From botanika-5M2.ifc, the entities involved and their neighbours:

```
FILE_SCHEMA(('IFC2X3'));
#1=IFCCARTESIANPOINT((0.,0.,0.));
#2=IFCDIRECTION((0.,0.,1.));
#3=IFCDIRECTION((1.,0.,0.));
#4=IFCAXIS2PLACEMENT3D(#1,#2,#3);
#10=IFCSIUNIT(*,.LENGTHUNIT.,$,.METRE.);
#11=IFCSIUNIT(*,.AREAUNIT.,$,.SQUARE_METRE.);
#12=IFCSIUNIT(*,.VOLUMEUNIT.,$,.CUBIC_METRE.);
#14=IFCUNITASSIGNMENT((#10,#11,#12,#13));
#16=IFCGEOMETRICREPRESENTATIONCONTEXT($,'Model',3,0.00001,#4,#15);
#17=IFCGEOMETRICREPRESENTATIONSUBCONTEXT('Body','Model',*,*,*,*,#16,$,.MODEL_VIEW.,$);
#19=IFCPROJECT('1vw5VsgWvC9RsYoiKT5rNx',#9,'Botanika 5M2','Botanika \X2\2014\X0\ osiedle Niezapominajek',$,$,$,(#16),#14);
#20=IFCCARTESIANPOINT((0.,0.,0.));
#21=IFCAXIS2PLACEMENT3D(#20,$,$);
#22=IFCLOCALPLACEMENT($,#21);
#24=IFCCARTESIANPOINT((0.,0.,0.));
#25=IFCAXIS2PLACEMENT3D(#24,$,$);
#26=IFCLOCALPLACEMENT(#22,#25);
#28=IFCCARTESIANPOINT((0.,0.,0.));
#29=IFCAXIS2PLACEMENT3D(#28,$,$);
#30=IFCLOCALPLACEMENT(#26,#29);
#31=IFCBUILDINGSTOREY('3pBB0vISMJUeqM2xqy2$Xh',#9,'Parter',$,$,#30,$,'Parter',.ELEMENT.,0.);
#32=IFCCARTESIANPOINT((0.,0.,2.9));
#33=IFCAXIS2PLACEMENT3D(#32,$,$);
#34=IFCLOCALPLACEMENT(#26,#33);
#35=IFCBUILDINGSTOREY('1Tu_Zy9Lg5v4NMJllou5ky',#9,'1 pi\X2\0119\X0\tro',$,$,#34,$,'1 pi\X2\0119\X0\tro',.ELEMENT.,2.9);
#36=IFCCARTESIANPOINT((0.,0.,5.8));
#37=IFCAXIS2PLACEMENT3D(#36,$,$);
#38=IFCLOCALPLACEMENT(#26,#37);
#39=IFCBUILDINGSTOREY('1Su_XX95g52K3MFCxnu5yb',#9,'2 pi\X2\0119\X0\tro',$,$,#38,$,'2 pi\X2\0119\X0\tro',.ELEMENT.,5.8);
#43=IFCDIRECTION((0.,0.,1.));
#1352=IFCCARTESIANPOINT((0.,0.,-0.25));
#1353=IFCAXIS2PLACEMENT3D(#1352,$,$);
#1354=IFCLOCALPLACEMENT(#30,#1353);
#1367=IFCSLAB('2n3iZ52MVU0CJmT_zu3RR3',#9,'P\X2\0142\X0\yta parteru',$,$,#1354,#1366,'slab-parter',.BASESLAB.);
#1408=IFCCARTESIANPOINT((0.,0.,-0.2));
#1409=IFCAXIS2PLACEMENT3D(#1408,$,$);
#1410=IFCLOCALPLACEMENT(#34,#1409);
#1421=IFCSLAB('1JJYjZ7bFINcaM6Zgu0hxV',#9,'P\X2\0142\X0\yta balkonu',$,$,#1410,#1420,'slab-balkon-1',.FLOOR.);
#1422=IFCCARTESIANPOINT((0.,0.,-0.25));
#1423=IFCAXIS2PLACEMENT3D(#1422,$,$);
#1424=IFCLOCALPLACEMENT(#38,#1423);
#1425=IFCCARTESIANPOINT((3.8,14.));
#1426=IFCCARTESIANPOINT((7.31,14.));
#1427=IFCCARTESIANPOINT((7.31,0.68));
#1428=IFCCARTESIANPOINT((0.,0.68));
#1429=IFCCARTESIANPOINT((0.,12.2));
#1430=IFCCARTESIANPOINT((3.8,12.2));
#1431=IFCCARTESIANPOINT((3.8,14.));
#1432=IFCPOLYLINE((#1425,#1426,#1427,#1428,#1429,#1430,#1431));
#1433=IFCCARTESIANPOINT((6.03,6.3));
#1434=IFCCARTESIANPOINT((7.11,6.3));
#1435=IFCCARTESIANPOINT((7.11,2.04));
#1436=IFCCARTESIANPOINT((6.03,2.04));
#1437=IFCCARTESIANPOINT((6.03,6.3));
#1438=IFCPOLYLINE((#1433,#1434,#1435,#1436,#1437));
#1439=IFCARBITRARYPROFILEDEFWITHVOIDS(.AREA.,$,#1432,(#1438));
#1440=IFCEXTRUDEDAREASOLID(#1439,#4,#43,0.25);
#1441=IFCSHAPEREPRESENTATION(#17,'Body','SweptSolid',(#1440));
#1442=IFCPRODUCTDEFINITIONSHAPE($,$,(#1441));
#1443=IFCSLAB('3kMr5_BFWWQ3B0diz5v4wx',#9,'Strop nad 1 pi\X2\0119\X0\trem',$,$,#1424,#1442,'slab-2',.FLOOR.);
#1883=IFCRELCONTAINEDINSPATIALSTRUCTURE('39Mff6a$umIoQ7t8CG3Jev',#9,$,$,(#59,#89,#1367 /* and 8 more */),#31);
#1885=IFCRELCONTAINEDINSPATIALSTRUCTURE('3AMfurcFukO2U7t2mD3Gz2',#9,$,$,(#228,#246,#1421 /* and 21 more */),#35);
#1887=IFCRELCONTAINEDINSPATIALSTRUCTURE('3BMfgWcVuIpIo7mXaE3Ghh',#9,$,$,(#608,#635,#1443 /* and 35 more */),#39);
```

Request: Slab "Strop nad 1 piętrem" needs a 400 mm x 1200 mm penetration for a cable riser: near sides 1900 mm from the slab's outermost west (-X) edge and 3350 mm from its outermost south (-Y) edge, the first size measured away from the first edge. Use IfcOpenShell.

```python
import numpy as np
import ifcopenshell
import ifcopenshell.api.feature
import ifcopenshell.api.geometry
import ifcopenshell.api.root
import ifcopenshell.geom
import ifcopenshell.util.placement
import ifcopenshell.util.representation
import ifcopenshell.util.shape
import ifcopenshell.util.unit

model = ifcopenshell.open("botanika-5M2.ifc")
unit_scale = ifcopenshell.util.unit.calculate_unit_scale(model)
settings = ifcopenshell.geom.settings()


def volume(element):
    """Net volume in cubic metres, openings subtracted."""
    shape = ifcopenshell.geom.create_shape(settings, element)
    return ifcopenshell.util.shape.get_volume(shape.geometry)


slab = model.by_guid("3kMr5_BFWWQ3B0diz5v4wx")
before = volume(slab)

# Extent in the slab's own axes, in metres. The edges named are its -X and -Y sides.
slab_shape = ifcopenshell.geom.create_shape(settings, slab)
vertices = ifcopenshell.util.shape.get_vertices(slab_shape.geometry)
x_min, y_min, bottom = vertices.min(axis=0)
top = vertices[:, 2].max()

opening = ifcopenshell.api.root.create_entity(model, ifc_class="IfcOpeningElement", name="Cable riser opening")
context = ifcopenshell.util.representation.get_context(model, "Model", "Body", "MODEL_VIEW")
width, depth = 0.4, 1.2
outline = [(0.0, 0.0), (width, 0.0), (width, depth), (0.0, depth), (0.0, 0.0)]
# Overshoot both faces by 50 mm so the cut is clean.
shape = ifcopenshell.api.geometry.add_slab_representation(
    model, context=context, depth=top - bottom + 0.1, polyline=outline
)
ifcopenshell.api.geometry.assign_representation(model, product=opening, representation=shape)

matrix = ifcopenshell.util.placement.get_local_placement(slab.ObjectPlacement)
matrix[:, 3] = matrix @ np.append(np.array([x_min + 1.9, y_min + 3.35, bottom - 0.05]) / unit_scale, 1.0)
ifcopenshell.api.geometry.edit_object_placement(model, product=opening, matrix=matrix, is_si=False)
ifcopenshell.api.feature.add_feature(model, feature=opening, element=slab)

after = volume(slab)

print(f"slab volume {before:.3f} -> {after:.3f} m3")

model.write("botanika-5M2_rev.ifc")
```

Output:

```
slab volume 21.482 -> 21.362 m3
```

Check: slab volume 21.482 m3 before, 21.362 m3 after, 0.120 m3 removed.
